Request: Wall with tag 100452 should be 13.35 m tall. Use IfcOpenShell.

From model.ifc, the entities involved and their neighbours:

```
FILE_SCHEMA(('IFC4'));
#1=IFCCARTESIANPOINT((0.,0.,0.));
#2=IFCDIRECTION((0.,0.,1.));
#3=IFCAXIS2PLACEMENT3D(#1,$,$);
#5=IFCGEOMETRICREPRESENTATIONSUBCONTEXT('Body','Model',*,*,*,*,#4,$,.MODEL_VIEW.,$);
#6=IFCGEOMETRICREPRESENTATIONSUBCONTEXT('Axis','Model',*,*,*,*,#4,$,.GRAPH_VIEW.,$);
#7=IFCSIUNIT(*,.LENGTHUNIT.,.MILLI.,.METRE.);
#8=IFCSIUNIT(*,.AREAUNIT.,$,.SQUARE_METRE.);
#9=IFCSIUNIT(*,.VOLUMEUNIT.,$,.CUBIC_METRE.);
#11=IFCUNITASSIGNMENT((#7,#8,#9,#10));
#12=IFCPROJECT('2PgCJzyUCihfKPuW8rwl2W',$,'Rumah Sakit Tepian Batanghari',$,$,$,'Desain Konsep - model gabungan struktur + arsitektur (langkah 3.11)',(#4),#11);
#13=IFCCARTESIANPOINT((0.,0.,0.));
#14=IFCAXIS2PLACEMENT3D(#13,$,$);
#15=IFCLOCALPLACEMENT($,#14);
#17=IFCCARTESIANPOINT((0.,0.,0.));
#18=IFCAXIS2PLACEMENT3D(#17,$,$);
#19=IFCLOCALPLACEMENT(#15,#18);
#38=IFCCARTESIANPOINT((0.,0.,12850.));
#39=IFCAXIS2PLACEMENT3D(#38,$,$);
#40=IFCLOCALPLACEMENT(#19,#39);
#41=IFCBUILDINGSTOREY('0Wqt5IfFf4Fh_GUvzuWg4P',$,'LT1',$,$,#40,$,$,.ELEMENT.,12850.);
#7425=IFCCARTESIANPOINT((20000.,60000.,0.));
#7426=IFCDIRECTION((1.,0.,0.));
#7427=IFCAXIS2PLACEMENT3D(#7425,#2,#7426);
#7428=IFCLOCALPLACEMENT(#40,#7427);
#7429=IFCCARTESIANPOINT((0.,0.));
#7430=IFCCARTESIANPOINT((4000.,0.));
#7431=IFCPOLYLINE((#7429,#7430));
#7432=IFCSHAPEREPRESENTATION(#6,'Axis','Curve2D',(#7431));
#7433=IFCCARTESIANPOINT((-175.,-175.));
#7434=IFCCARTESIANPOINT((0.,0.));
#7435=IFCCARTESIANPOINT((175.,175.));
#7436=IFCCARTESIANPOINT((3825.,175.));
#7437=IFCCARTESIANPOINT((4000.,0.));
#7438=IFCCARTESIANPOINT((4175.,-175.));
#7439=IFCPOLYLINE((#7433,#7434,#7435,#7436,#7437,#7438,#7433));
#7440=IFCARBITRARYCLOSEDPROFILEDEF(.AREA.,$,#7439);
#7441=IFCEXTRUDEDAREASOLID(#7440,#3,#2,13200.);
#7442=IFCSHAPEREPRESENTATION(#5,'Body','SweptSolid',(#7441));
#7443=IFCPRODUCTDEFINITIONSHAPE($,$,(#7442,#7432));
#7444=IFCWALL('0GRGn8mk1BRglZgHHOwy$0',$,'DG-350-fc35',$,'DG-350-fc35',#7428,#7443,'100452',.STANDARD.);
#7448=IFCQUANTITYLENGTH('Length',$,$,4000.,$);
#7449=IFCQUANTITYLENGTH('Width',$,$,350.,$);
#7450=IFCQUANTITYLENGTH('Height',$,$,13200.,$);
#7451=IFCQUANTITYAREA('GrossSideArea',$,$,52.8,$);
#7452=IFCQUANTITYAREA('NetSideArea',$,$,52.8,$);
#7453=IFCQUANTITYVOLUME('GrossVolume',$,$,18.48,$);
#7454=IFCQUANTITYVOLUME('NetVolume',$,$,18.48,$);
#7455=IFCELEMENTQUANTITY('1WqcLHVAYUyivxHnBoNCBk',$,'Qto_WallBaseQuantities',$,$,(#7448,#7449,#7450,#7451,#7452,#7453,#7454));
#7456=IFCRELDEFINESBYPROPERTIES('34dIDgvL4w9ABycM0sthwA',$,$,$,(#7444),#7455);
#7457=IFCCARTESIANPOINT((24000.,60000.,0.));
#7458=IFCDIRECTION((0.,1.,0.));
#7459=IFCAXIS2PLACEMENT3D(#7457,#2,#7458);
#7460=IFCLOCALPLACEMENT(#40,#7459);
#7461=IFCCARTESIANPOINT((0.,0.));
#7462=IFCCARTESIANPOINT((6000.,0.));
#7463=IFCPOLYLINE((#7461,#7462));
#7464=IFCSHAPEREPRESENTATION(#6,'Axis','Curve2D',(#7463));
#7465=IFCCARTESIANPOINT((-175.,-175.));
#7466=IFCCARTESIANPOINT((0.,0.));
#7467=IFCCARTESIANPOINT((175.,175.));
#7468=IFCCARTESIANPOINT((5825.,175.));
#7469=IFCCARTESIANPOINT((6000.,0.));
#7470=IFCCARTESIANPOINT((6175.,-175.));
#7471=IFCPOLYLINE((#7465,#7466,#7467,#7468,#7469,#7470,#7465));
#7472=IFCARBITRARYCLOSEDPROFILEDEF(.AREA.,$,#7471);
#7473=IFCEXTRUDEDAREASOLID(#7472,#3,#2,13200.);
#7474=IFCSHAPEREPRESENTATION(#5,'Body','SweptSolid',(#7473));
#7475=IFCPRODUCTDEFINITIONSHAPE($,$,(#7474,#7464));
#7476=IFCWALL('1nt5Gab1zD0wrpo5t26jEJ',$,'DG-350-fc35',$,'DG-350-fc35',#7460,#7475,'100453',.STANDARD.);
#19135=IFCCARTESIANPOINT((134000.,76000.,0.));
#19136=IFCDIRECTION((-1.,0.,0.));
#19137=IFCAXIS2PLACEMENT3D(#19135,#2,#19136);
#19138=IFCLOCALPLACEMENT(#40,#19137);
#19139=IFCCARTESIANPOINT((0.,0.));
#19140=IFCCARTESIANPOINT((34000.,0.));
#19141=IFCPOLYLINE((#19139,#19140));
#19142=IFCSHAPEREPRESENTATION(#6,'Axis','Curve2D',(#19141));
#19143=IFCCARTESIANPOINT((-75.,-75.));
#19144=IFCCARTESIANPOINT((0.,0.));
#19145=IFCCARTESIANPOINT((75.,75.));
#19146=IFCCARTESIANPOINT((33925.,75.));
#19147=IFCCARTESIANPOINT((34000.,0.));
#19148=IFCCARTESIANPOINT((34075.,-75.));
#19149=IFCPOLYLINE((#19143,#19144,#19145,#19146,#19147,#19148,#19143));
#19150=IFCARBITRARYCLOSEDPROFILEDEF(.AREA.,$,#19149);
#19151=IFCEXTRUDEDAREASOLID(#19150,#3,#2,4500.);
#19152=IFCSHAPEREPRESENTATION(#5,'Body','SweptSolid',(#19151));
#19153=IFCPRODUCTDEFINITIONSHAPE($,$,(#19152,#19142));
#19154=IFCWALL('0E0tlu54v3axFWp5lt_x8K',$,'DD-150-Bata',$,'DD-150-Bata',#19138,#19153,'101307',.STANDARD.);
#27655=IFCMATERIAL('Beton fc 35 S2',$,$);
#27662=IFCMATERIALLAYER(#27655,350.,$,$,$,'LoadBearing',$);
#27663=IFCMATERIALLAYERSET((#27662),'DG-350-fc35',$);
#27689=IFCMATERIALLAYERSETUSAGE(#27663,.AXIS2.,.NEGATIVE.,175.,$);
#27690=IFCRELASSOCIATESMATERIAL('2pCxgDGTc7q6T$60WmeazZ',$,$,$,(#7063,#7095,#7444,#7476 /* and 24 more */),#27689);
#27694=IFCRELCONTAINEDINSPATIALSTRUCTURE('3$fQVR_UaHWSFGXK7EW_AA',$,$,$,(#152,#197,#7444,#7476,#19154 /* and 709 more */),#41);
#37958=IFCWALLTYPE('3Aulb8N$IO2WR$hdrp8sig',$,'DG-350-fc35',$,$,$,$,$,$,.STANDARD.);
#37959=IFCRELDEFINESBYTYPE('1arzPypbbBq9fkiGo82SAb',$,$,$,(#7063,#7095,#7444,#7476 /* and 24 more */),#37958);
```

```python
import ifcopenshell
import ifcopenshell.api.pset
import ifcopenshell.geom
import ifcopenshell.util.element
import ifcopenshell.util.representation
import ifcopenshell.util.shape
import ifcopenshell.util.unit

model = ifcopenshell.open("model.ifc")
unit_scale = ifcopenshell.util.unit.calculate_unit_scale(model)
area_scale = ifcopenshell.util.unit.calculate_unit_scale(model, "AREAUNIT")
volume_scale = ifcopenshell.util.unit.calculate_unit_scale(model, "VOLUMEUNIT")
settings = ifcopenshell.geom.settings()


def volume(element):
    """Net volume in cubic metres, openings subtracted."""
    shape = ifcopenshell.geom.create_shape(settings, element)
    return ifcopenshell.util.shape.get_volume(shape.geometry)


wall = model.by_id(7444)
before = volume(wall)

body = ifcopenshell.util.representation.get_representation(wall, "Model", "Body")
solid = body.Items[0]
old_height = solid.Depth
solid.Depth = 13.35 / unit_scale
after = volume(wall)
thickness = 0.35  # wall thickness in metres

# Update the stored height, areas and volumes.
qto = model.by_id(ifcopenshell.util.element.get_pset(wall, "Qto_WallBaseQuantities", should_inherit=False)["id"])
ifcopenshell.api.pset.edit_qto(model, qto=qto, properties={
    "Height": solid.Depth,
    "GrossSideArea": ifcopenshell.util.element.get_pset(wall, "Qto_WallBaseQuantities", "GrossSideArea") * solid.Depth / old_height,
    "NetSideArea": after / thickness / area_scale,
    "GrossVolume": ifcopenshell.util.element.get_pset(wall, "Qto_WallBaseQuantities", "GrossVolume") * solid.Depth / old_height,
    "NetVolume": after / volume_scale,
})

print(f"height {old_height:g} -> {solid.Depth:g}, volume {before:.3f} -> {after:.3f} m3")

model.write("model_updated.ifc")
```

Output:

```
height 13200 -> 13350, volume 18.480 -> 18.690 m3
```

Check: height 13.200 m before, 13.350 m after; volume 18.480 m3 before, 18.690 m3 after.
